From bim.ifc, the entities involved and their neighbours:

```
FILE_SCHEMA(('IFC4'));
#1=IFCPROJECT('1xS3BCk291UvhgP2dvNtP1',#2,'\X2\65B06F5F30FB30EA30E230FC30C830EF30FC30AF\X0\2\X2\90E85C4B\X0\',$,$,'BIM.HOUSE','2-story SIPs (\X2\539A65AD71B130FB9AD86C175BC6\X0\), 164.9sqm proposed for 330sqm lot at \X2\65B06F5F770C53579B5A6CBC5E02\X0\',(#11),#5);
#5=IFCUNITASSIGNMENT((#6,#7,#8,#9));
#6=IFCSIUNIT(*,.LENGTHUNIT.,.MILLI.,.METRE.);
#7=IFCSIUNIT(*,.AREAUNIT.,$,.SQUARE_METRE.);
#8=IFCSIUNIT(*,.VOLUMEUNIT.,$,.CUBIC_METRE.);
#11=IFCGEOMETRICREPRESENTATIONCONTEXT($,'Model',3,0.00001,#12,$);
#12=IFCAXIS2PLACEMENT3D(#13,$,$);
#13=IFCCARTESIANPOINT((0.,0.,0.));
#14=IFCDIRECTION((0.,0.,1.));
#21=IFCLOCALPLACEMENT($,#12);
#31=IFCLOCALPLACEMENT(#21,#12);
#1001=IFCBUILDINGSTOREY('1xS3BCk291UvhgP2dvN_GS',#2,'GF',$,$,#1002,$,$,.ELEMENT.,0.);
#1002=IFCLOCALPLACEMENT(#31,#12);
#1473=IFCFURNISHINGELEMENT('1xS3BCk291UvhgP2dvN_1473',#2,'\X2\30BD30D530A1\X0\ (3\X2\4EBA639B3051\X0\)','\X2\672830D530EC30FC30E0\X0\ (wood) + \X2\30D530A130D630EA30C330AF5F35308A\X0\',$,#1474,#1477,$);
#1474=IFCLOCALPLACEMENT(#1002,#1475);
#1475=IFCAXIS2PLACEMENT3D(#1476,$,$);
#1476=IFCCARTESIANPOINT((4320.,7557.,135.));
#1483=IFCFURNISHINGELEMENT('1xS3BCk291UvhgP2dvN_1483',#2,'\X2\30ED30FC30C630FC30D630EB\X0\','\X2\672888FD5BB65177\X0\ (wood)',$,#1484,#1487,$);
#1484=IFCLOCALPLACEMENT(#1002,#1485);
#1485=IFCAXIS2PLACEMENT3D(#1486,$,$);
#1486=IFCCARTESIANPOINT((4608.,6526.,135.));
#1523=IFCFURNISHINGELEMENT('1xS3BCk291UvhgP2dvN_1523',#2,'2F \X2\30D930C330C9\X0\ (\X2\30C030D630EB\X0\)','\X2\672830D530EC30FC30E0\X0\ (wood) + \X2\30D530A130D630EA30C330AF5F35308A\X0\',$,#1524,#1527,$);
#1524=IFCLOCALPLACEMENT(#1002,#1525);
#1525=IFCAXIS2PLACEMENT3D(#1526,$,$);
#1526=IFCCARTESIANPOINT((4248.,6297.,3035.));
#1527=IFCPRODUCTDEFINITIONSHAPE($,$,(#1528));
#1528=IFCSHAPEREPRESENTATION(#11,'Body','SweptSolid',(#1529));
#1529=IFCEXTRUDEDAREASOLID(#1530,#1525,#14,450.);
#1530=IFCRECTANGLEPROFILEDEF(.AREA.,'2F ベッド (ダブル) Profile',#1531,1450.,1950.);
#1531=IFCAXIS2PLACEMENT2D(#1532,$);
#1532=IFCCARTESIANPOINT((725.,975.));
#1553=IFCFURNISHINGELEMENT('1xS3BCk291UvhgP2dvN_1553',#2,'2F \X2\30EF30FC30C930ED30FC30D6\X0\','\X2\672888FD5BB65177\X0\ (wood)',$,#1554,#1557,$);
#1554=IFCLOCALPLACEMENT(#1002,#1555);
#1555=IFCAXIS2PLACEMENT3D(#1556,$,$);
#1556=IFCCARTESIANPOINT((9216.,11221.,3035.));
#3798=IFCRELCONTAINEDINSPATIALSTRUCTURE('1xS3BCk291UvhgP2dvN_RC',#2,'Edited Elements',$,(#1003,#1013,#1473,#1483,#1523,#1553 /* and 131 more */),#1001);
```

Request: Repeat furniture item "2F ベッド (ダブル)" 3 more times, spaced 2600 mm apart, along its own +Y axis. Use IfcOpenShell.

```python
import ifcopenshell
import ifcopenshell.api.geometry
import ifcopenshell.api.root
import ifcopenshell.util.element
import ifcopenshell.util.placement
import ifcopenshell.util.unit

model = ifcopenshell.open("bim.ifc")
unit_scale = ifcopenshell.util.unit.calculate_unit_scale(model)


def reuse_history(source, copy):
    """copy_class also copies each property set's owner history, people and application; keep the originals."""
    for rel in copy.IsDefinedBy:
        if rel.is_a("IfcRelDefinesByProperties") and (history := rel.RelatingPropertyDefinition.OwnerHistory):
            rel.RelatingPropertyDefinition.OwnerHistory = source.OwnerHistory
            ifcopenshell.util.element.remove_deep2(model, history)


source = model.by_id(1523)
base = ifcopenshell.util.placement.get_local_placement(source.ObjectPlacement)
step = base[:3, 1] * 2.6 / unit_scale

for i in range(1, 4):
    copy = ifcopenshell.api.root.copy_class(model, product=source)
    copy.Representation = ifcopenshell.util.element.copy_deep(
        model, source.Representation, exclude=["IfcGeometricRepresentationContext", "IfcRepresentationMap"]
    )
    reuse_history(source, copy)
    matrix = base.copy()
    matrix[:3, 3] += i * step
    print("added at", matrix[:3, 3].round(3) + 0.0)
    ifcopenshell.api.geometry.edit_object_placement(model, product=copy, matrix=matrix, is_si=False)

model.write("bim-out.ifc")
```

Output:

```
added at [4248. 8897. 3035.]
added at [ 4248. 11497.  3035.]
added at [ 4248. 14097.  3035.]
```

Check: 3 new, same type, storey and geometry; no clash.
